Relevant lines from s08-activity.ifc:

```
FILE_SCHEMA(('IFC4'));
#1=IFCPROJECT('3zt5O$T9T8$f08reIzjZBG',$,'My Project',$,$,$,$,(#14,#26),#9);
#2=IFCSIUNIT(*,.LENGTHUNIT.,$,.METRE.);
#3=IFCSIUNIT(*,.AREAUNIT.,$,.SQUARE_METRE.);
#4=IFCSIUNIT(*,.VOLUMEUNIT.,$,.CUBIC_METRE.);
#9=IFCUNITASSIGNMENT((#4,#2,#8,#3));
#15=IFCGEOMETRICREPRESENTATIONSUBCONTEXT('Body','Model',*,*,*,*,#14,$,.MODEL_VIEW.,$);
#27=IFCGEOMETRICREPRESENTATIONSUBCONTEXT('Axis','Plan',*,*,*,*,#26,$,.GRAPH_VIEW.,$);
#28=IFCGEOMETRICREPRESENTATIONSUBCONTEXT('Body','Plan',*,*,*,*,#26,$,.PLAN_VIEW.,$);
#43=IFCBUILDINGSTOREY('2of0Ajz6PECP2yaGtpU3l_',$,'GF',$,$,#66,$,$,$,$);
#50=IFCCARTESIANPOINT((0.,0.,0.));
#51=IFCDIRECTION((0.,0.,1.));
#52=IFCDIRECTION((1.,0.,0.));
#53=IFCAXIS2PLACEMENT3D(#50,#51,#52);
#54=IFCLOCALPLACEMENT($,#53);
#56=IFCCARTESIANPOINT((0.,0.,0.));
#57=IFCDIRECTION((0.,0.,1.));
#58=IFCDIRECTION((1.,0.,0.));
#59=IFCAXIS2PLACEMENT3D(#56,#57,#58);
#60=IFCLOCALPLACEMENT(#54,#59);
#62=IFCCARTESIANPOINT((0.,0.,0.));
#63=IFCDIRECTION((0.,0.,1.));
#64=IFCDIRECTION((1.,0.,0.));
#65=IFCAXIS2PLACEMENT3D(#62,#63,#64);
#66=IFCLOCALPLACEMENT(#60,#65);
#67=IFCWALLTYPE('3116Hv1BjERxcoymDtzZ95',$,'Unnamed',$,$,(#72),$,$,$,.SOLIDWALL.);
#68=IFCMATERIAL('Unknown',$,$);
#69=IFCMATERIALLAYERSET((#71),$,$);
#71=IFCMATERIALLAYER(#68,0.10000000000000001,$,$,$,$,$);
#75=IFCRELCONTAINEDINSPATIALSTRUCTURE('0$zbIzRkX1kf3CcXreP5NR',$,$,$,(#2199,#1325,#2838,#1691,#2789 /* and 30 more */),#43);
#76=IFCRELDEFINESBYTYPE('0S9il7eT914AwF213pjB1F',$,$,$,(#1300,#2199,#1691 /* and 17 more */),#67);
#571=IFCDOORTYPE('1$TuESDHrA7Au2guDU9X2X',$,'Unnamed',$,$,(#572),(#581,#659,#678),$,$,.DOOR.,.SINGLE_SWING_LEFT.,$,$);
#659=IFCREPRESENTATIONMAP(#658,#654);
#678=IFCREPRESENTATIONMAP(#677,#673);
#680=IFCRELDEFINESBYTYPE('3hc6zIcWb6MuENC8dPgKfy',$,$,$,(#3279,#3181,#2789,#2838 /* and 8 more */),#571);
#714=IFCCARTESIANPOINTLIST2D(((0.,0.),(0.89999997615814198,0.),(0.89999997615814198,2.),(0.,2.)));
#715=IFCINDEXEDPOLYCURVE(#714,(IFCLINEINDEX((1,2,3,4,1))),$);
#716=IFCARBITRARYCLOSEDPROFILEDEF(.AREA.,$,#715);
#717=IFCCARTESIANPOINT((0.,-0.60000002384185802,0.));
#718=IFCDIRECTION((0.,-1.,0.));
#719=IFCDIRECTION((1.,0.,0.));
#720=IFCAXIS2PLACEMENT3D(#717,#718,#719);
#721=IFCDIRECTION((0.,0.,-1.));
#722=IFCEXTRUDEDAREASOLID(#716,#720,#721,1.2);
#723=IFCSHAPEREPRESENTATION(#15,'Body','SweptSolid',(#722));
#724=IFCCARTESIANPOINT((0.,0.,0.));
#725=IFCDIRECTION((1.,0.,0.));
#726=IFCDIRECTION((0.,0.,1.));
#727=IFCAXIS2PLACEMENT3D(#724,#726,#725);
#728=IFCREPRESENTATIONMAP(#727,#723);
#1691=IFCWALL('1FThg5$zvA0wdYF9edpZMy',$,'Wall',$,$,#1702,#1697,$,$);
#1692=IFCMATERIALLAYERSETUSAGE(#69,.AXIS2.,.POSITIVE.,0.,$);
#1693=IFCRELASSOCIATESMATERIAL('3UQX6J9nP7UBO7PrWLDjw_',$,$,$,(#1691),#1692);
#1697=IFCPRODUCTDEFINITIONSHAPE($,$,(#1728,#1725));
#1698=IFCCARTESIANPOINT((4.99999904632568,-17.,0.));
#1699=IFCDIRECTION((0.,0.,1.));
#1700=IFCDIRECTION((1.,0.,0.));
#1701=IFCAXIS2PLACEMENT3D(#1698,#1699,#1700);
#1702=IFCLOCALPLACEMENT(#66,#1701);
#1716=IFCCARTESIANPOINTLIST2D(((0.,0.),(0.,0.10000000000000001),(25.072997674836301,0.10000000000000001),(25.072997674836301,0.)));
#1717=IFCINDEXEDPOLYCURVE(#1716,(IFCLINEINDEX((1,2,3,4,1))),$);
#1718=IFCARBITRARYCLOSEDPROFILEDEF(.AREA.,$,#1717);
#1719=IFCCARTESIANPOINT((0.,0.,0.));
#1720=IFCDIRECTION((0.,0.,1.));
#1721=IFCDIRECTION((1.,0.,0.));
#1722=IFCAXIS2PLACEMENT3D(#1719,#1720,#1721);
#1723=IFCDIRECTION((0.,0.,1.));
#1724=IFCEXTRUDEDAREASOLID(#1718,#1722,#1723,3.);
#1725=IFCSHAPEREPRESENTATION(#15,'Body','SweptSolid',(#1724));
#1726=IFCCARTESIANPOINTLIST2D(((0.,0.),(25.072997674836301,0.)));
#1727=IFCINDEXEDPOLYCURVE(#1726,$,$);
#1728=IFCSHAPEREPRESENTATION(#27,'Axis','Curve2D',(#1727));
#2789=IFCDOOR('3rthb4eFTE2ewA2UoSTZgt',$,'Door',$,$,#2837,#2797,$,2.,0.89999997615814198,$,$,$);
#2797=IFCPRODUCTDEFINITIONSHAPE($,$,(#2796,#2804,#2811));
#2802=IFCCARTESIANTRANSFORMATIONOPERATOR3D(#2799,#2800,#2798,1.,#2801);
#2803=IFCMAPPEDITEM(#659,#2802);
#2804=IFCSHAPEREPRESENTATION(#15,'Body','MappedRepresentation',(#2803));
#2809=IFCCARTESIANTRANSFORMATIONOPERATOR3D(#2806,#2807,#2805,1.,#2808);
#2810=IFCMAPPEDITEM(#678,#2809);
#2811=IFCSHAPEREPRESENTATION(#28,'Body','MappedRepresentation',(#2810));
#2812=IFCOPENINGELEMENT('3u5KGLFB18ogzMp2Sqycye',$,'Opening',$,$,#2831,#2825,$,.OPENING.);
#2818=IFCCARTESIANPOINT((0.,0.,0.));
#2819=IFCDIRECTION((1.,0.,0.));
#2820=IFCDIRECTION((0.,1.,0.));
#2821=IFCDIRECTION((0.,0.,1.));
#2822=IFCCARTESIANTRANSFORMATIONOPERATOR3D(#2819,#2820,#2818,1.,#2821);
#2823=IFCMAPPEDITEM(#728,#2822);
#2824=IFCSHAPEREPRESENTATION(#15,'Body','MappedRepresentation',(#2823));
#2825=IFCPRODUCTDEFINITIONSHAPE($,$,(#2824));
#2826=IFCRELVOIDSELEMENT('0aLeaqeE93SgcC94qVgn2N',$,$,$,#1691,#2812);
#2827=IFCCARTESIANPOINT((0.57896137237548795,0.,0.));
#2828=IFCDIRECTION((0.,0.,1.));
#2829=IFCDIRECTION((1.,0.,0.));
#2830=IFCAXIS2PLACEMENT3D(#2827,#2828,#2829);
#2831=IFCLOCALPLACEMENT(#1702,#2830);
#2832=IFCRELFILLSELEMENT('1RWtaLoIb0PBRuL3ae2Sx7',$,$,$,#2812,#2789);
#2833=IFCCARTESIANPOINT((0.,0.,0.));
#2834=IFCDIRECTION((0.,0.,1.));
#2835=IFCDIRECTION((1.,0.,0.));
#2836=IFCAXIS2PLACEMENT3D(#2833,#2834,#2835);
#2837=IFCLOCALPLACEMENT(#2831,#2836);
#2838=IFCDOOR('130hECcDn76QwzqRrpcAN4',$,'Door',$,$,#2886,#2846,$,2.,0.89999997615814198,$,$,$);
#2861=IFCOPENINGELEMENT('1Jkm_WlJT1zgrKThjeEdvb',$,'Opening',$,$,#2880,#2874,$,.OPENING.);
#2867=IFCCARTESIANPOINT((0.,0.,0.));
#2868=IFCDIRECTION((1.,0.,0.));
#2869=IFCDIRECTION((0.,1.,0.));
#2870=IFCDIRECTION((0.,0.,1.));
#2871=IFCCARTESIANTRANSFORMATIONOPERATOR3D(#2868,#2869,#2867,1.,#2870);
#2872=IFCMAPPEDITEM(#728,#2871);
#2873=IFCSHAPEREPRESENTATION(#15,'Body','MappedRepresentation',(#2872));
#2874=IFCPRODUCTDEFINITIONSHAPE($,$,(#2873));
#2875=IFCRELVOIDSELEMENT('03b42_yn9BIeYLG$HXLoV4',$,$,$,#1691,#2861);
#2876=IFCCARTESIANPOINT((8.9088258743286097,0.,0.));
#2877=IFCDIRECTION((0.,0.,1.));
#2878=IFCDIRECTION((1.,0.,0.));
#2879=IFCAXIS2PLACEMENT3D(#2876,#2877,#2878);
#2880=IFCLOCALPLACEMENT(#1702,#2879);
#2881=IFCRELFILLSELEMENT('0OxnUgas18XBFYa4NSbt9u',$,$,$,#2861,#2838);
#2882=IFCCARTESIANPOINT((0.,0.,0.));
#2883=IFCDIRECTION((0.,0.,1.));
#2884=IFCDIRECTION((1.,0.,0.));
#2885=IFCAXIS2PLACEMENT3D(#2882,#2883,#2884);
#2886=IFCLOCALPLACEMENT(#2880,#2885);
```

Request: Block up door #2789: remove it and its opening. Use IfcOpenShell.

```python
import ifcopenshell
import ifcopenshell.api.feature
import ifcopenshell.api.root
import ifcopenshell.geom
import ifcopenshell.util.shape

model = ifcopenshell.open("s08-activity.ifc")
settings = ifcopenshell.geom.settings()


def volume(element):
    """Net volume in cubic metres, openings subtracted."""
    shape = ifcopenshell.geom.create_shape(settings, element)
    return ifcopenshell.util.shape.get_volume(shape.geometry)


door = model.by_guid("3rthb4eFTE2ewA2UoSTZgt")
opening = door.FillsVoids[0].RelatingOpeningElement
wall = opening.VoidsElements[0].RelatingBuildingElement
before = volume(wall)

ifcopenshell.api.root.remove_product(model, product=door)
ifcopenshell.api.feature.remove_feature(model, feature=opening)

after = volume(wall)

print(f"wall volume {before:.3f} -> {after:.3f} m3")

model.write("s08-activity-out.ifc")
```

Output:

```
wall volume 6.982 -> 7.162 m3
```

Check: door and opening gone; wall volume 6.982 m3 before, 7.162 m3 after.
